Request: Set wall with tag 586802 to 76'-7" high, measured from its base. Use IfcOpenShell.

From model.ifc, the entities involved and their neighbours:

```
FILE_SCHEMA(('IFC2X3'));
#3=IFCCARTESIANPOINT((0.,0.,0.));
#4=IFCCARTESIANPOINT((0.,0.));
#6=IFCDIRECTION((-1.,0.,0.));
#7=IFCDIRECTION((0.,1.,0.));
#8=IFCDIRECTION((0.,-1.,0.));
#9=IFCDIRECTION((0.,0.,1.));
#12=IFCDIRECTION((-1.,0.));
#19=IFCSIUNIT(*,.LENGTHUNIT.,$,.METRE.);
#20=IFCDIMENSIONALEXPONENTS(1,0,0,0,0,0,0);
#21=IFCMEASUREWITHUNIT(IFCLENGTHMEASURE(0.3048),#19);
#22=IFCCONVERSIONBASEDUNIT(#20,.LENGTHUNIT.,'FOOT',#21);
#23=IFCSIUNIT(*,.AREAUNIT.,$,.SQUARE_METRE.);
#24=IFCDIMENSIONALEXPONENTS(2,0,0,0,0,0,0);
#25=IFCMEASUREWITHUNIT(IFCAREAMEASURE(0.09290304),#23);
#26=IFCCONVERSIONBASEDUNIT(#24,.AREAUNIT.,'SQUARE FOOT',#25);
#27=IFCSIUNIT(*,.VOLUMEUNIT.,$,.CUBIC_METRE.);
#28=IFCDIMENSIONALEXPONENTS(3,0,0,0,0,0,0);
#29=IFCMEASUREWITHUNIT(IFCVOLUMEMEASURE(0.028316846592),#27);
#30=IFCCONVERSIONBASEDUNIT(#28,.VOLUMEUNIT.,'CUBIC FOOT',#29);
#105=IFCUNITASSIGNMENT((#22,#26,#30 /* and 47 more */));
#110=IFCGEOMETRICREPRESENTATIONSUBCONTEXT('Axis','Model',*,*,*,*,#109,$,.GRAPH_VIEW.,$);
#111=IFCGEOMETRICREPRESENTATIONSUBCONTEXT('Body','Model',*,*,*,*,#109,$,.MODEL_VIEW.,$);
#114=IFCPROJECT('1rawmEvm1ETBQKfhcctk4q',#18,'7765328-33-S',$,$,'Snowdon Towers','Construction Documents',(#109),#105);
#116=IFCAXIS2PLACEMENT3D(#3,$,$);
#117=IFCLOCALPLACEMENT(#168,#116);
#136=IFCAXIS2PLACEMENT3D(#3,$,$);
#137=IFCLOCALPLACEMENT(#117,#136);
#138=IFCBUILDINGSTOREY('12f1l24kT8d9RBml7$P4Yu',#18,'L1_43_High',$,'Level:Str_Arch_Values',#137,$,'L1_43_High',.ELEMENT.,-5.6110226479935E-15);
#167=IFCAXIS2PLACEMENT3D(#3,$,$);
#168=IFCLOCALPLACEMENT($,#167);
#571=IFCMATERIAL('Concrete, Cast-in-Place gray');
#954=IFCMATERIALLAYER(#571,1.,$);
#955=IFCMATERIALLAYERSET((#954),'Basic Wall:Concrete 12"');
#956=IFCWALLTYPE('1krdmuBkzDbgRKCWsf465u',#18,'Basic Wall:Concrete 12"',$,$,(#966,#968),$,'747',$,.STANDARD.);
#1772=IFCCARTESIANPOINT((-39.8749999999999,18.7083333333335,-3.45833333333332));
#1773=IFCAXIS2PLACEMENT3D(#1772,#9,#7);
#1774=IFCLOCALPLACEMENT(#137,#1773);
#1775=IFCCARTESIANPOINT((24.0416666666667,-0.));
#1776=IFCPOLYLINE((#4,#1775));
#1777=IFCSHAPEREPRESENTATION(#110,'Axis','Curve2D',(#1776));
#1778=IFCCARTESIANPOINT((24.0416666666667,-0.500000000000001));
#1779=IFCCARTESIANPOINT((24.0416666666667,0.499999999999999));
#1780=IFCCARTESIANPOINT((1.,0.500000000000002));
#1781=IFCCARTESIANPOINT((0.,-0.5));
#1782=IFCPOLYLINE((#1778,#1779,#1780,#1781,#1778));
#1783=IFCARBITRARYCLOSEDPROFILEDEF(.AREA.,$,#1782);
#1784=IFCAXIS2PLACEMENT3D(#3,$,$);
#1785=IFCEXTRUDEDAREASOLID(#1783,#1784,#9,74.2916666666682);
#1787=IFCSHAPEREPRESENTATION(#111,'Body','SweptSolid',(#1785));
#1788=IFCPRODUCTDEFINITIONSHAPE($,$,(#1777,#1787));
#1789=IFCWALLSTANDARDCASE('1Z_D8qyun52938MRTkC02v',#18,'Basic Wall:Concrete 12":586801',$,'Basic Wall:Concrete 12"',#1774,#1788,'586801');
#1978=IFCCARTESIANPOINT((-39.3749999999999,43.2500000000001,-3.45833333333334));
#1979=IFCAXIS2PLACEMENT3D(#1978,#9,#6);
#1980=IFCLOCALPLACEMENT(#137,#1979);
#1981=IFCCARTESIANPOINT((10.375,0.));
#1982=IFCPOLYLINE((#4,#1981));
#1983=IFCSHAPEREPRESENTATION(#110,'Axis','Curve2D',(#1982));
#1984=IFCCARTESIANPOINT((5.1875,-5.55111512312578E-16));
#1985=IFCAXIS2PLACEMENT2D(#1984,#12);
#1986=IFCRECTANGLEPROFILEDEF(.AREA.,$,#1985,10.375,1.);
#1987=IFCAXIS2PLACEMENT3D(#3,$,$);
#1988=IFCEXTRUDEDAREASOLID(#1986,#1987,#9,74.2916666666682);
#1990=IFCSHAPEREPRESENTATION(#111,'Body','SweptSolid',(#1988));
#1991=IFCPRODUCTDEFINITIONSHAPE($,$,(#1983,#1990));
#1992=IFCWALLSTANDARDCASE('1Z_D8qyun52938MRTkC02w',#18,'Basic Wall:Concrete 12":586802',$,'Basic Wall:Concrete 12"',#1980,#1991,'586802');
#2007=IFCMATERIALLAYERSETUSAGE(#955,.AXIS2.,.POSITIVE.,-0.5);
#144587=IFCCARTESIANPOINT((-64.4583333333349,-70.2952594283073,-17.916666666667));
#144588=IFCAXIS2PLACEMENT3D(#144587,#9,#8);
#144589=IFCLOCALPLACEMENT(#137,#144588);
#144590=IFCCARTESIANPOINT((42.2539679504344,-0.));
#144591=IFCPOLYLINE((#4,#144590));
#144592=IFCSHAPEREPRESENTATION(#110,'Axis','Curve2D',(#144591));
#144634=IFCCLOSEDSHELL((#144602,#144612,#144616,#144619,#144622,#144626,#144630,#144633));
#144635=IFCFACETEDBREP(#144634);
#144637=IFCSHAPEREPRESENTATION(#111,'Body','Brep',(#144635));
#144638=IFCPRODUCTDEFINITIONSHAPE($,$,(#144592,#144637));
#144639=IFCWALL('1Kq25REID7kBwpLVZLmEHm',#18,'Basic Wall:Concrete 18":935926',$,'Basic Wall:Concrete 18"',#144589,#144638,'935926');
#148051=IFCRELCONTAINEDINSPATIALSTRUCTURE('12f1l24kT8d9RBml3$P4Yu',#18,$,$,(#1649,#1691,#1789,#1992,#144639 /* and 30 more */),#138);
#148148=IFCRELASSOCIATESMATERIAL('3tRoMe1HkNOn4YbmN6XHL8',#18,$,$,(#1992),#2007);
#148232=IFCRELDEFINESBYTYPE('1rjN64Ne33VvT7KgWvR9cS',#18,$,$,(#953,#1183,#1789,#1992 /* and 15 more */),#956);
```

```python
import ifcopenshell
import ifcopenshell.geom
import ifcopenshell.util.representation
import ifcopenshell.util.shape
import ifcopenshell.util.unit

model = ifcopenshell.open("model.ifc")
unit_scale = ifcopenshell.util.unit.calculate_unit_scale(model)
settings = ifcopenshell.geom.settings()


def volume(element):
    """Net volume in cubic metres, openings subtracted."""
    shape = ifcopenshell.geom.create_shape(settings, element)
    return ifcopenshell.util.shape.get_volume(shape.geometry)


wall = model.by_guid("1Z_D8qyun52938MRTkC02w")
before = volume(wall)

body = ifcopenshell.util.representation.get_representation(wall, "Model", "Body")
solid = body.Items[0]
old_height = solid.Depth
solid.Depth = 919 * 0.0254 / unit_scale
after = volume(wall)

print(f"height {old_height:g} -> {solid.Depth:g}, volume {before:.3f} -> {after:.3f} m3")

model.write("model_rev.ifc")
```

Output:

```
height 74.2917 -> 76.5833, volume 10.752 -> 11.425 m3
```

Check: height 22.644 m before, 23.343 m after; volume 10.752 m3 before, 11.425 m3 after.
